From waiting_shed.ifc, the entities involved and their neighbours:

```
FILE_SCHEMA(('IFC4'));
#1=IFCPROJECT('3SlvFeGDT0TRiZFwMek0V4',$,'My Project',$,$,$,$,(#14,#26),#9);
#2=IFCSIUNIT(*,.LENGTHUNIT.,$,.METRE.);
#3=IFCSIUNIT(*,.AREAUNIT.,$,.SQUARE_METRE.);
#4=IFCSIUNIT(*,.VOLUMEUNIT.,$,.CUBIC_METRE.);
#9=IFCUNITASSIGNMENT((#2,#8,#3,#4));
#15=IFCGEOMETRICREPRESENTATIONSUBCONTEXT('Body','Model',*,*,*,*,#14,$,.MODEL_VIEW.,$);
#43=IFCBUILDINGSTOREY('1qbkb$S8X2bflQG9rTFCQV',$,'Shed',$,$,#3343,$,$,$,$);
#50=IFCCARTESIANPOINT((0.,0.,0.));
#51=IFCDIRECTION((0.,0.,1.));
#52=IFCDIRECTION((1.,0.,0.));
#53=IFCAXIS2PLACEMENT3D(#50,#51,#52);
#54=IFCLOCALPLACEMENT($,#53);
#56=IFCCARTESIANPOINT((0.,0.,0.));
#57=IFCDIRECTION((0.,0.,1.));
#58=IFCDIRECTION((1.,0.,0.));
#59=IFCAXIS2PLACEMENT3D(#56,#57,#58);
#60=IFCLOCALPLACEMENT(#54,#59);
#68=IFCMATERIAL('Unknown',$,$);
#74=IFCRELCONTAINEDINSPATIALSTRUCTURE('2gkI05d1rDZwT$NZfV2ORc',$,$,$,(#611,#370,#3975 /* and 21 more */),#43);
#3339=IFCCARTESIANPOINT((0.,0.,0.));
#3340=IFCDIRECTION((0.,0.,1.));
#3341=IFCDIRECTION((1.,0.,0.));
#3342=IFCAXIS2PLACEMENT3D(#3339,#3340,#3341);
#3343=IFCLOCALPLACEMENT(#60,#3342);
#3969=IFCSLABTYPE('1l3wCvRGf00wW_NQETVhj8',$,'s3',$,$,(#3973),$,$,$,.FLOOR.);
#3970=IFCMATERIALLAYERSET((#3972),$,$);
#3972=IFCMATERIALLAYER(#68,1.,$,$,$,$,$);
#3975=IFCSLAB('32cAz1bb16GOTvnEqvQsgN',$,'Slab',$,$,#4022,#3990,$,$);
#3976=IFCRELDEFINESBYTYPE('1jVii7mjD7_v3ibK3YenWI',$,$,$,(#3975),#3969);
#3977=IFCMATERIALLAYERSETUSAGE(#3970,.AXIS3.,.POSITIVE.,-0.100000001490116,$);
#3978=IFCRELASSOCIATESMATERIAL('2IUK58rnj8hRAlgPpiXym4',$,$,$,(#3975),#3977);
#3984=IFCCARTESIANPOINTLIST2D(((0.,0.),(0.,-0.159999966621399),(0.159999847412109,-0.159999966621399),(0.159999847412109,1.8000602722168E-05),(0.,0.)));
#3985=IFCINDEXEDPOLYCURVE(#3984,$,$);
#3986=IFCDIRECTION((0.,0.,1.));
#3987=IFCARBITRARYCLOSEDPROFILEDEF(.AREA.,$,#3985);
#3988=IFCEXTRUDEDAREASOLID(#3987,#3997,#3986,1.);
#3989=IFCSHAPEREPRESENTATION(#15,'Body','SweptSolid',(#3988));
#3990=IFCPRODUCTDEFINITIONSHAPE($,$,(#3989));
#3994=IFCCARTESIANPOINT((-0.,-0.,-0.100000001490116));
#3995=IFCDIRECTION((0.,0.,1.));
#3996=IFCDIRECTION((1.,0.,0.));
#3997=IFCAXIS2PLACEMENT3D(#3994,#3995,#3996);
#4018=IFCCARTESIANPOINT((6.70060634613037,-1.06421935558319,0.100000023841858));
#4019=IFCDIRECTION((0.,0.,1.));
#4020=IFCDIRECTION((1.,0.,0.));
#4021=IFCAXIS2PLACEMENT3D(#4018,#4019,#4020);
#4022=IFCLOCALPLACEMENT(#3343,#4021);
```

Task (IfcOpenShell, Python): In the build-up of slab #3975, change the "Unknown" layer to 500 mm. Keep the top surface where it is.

```python
import ifcopenshell
import ifcopenshell.util.element
import ifcopenshell.util.representation
import ifcopenshell.util.unit

model = ifcopenshell.open("waiting_shed.ifc")
unit_scale = ifcopenshell.util.unit.calculate_unit_scale(model)

layer_set = model.by_id(3970)
layer = next(l for l in layer_set.MaterialLayers if l.Material and l.Material.Name == "Unknown")
change = 0.5 / unit_scale - layer.LayerThickness
layer.LayerThickness += change

# Geometry does not follow the layer set by itself.
slabs = [e for e in ifcopenshell.util.element.get_elements_by_material(model, layer_set) if e.is_a("IfcSlab")]
for slab in sorted(slabs, key=lambda e: e.id()):
    body = ifcopenshell.util.representation.get_representation(slab, "Model", "Body")
    solid = body.Items[0]
    old_depth = solid.Depth
    solid.Depth += change
    # Extruded upwards: lower the start of the extrusion so the top stays.
    x, y, z = solid.Position.Location.Coordinates
    solid.Position.Location = model.createIfcCartesianPoint((x, y, z - change))
    print(slab.id(), f"{old_depth:g} -> {solid.Depth:g}")

# The layers are counted up from the underside, which has moved.
for usage in {ifcopenshell.util.element.get_material(slab) for slab in slabs}:
    usage.OffsetFromReferenceLine -= change

model.write("waiting_shed_edited.ifc")
```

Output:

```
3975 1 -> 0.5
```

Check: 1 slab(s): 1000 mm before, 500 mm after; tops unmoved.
